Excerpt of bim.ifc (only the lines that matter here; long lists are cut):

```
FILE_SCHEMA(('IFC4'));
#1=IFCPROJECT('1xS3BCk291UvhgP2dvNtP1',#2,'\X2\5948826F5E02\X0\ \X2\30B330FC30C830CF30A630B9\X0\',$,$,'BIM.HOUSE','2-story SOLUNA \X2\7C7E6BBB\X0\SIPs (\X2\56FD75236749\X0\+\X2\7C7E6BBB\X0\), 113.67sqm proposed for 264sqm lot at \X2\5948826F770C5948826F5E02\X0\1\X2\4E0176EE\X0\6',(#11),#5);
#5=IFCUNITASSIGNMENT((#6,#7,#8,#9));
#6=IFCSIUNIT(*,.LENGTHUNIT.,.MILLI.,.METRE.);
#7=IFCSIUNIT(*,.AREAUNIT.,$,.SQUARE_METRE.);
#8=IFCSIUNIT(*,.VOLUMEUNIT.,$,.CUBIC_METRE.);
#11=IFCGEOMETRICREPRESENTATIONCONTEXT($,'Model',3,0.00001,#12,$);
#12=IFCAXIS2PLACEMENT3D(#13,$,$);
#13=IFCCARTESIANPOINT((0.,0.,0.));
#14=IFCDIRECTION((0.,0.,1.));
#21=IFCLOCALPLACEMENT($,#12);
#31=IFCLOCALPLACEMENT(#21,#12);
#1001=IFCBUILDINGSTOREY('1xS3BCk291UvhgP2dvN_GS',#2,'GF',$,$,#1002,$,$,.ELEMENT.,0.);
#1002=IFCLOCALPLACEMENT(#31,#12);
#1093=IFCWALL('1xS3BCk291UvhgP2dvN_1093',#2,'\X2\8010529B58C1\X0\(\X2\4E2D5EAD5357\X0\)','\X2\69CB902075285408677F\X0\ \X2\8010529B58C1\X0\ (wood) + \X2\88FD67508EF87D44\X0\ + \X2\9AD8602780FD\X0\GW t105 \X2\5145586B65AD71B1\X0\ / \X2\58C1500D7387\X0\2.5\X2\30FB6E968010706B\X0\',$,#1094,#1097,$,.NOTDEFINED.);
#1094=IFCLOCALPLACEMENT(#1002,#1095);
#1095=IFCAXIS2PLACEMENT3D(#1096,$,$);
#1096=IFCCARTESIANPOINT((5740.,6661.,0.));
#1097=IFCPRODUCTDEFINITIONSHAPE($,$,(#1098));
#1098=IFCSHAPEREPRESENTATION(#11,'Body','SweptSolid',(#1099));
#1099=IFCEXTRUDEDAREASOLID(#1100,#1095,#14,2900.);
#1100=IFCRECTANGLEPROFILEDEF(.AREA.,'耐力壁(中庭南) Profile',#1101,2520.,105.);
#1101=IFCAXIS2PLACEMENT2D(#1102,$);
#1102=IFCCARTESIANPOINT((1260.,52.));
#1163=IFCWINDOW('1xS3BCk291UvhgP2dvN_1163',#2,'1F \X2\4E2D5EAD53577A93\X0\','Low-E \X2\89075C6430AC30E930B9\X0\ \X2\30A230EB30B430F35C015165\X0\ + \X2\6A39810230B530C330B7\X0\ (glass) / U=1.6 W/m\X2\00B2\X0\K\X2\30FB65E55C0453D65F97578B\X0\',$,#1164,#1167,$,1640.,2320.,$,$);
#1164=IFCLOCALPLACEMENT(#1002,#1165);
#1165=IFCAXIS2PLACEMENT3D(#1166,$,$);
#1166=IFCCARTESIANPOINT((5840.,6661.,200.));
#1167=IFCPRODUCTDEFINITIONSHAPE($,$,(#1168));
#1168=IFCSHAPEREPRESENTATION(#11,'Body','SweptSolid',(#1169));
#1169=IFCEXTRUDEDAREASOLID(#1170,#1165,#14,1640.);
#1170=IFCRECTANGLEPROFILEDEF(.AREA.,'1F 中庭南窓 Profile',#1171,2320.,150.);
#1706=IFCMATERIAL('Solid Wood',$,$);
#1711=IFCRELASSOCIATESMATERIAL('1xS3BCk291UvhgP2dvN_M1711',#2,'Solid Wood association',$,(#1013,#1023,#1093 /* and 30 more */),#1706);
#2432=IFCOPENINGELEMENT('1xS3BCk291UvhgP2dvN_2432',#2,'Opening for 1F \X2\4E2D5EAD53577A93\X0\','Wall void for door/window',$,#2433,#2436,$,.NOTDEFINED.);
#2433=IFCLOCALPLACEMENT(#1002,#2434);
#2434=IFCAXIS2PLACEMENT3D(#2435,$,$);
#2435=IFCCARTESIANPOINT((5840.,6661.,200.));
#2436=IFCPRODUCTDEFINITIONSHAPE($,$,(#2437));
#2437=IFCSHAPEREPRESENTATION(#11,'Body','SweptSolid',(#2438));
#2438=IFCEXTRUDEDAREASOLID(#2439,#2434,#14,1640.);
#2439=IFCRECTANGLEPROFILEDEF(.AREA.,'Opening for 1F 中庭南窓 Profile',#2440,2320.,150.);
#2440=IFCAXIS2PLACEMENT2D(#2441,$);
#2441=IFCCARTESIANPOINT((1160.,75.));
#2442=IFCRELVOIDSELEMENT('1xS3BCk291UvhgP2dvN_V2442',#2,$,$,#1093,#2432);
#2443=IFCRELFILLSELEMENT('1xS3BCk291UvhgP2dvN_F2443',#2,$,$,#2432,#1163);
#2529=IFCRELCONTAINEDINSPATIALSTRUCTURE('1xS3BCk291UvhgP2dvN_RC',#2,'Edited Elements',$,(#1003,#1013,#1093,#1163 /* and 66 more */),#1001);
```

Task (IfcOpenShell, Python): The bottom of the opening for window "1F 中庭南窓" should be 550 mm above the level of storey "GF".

```python
import numpy as np
import ifcopenshell
import ifcopenshell.api.geometry
import ifcopenshell.geom
import ifcopenshell.util.element
import ifcopenshell.util.placement
import ifcopenshell.util.shape
import ifcopenshell.util.unit

model = ifcopenshell.open("bim.ifc")
unit_scale = ifcopenshell.util.unit.calculate_unit_scale(model)

window = model.by_guid("1xS3BCk291UvhgP2dvN_1163")
opening = window.FillsVoids[0].RelatingOpeningElement
storey = ifcopenshell.util.element.get_container(window, ifc_class="IfcBuildingStorey")
level = ifcopenshell.util.placement.get_local_placement(storey.ObjectPlacement)[2, 3]

# The opening's origin need not be at the sill, so measure its lowest point.
shape = ifcopenshell.geom.create_shape(ifcopenshell.geom.settings(), opening)
bottom = ifcopenshell.util.shape.get_shape_bottom_elevation(shape, shape.geometry) / unit_scale
dz = level + 550.0 - bottom

shift = np.array([0.0, 0.0, dz])
# The window is not placed relative to its opening, so move both.
for product in (opening, window):
    matrix = ifcopenshell.util.placement.get_local_placement(product.ObjectPlacement)
    matrix[:3, 3] += shift
    ifcopenshell.api.geometry.edit_object_placement(model, product=product, matrix=matrix, is_si=False)

print(f"moved by {dz * unit_scale:+.3f} m")

model.write("bim_edited.ifc")
```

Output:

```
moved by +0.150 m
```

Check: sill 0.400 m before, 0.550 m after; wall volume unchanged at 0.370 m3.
